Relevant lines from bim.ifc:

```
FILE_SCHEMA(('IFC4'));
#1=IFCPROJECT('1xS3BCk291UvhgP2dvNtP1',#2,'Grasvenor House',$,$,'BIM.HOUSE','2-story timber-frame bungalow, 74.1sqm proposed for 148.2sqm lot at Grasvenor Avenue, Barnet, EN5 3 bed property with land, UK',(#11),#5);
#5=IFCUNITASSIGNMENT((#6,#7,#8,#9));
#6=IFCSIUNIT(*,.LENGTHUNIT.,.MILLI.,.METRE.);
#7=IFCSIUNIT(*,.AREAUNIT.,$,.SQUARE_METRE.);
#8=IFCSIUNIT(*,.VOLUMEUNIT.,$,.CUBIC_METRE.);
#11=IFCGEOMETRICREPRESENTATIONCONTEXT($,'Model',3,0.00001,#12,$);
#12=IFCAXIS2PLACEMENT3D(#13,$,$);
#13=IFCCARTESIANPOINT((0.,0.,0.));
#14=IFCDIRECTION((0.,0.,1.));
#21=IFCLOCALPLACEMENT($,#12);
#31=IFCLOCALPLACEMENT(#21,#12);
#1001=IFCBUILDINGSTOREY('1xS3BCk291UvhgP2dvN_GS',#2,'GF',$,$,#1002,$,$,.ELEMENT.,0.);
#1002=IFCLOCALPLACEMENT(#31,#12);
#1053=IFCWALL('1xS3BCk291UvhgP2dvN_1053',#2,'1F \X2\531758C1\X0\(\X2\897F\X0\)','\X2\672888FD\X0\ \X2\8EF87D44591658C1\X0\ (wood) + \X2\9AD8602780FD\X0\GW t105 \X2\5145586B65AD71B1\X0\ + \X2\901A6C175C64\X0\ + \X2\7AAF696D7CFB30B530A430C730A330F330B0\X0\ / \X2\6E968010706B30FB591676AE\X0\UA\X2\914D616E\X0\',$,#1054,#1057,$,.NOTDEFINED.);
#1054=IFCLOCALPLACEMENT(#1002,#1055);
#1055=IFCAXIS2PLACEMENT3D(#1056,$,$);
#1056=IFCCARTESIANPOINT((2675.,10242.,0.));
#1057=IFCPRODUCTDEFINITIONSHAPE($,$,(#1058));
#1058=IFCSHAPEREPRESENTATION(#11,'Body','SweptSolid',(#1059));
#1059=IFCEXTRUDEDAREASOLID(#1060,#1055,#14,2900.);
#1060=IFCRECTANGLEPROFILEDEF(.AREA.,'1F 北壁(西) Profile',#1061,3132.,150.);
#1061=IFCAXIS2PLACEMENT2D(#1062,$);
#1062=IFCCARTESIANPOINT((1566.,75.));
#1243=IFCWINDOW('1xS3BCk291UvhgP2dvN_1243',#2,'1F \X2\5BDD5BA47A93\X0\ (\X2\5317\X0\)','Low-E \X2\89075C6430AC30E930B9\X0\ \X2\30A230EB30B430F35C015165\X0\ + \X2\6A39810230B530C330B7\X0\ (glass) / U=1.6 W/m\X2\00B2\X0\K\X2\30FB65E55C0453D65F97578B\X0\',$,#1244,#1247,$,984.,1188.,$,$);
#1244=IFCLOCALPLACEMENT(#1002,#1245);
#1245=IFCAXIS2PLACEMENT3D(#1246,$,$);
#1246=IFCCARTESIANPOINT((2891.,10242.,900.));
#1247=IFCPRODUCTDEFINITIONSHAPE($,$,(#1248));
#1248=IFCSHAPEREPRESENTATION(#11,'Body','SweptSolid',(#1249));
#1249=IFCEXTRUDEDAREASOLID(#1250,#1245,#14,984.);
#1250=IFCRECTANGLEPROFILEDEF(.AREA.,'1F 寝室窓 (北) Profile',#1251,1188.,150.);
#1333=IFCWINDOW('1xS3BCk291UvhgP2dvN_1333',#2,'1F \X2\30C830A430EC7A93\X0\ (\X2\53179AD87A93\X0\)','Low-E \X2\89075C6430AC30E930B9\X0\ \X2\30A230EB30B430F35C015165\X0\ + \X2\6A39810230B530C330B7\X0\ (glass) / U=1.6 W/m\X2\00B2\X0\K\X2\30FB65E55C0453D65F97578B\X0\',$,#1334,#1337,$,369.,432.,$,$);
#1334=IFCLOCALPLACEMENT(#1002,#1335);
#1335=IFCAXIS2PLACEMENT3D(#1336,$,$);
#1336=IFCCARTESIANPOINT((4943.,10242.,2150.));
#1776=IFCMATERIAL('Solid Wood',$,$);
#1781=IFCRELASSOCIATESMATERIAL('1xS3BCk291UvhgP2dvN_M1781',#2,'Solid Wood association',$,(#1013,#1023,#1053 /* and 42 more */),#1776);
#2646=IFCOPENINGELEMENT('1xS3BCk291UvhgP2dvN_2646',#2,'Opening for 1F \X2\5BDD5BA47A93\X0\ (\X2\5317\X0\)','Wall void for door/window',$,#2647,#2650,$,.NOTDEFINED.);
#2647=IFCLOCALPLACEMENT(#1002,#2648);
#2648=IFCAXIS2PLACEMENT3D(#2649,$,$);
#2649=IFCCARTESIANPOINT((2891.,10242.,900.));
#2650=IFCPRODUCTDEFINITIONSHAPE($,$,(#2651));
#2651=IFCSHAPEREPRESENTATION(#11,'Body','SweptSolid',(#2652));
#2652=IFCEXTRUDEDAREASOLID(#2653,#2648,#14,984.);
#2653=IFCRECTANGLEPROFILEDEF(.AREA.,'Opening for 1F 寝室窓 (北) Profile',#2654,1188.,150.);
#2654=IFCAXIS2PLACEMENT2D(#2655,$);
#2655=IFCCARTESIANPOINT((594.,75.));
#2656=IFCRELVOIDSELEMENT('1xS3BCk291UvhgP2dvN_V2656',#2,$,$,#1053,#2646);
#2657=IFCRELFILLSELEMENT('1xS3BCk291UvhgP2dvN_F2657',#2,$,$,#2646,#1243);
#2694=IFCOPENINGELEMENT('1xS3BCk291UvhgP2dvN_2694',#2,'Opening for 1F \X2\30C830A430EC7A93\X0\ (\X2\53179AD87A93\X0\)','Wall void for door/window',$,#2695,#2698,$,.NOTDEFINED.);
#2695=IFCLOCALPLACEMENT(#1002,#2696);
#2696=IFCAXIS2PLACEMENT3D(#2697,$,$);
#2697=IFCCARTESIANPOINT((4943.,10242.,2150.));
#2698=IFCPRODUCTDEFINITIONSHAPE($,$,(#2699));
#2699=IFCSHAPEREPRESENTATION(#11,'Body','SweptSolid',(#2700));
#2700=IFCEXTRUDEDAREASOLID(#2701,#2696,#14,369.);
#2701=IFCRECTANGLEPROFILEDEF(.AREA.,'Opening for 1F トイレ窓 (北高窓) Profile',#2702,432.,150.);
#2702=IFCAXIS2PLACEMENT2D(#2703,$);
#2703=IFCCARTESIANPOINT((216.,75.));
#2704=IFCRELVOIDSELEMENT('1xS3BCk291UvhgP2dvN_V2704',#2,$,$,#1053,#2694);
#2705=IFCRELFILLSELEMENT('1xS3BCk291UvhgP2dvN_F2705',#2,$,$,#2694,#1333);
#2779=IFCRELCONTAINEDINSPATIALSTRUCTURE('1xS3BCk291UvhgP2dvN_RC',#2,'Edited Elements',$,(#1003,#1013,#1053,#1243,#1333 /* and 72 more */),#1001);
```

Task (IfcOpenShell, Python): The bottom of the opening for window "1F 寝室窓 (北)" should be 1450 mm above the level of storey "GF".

```python
import numpy as np
import ifcopenshell
import ifcopenshell.api.geometry
import ifcopenshell.geom
import ifcopenshell.util.element
import ifcopenshell.util.placement
import ifcopenshell.util.shape
import ifcopenshell.util.unit

model = ifcopenshell.open("bim.ifc")
unit_scale = ifcopenshell.util.unit.calculate_unit_scale(model)

window = model.by_guid("1xS3BCk291UvhgP2dvN_1243")
opening = window.FillsVoids[0].RelatingOpeningElement
storey = ifcopenshell.util.element.get_container(window, ifc_class="IfcBuildingStorey")
level = ifcopenshell.util.placement.get_local_placement(storey.ObjectPlacement)[2, 3]

# The opening's origin need not be at the sill, so measure its lowest point.
shape = ifcopenshell.geom.create_shape(ifcopenshell.geom.settings(), opening)
bottom = ifcopenshell.util.shape.get_shape_bottom_elevation(shape, shape.geometry) / unit_scale
dz = level + 1450.0 - bottom

shift = np.array([0.0, 0.0, dz])
# The window is not placed relative to its opening, so move both.
for product in (opening, window):
    matrix = ifcopenshell.util.placement.get_local_placement(product.ObjectPlacement)
    matrix[:3, 3] += shift
    ifcopenshell.api.geometry.edit_object_placement(model, product=product, matrix=matrix, is_si=False)

print(f"moved by {dz * unit_scale:+.3f} m")

model.write("bim_rev.ifc")
```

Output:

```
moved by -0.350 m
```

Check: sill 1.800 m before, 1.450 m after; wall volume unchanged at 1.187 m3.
